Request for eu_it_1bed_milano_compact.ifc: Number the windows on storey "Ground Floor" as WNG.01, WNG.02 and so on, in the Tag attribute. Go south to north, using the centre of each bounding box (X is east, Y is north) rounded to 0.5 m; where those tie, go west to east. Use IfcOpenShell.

First a look at what the model holds.

```python
import ifcopenshell
import ifcopenshell.util.element
import ifcopenshell.util.placement

model = ifcopenshell.open("eu_it_1bed_milano_compact.ifc")
print(model.schema)
storey = next(s for s in model.by_type("IfcBuildingStorey") if s.Name == "Ground Floor")
windows = [e for e in ifcopenshell.util.element.get_decomposition(storey) if e.is_a("IfcWindow")]
for e in sorted(windows, key=lambda e: e.id()):
    origin = ifcopenshell.util.placement.get_local_placement(e.ObjectPlacement)[:3, 3]
    print(e.id(), e.Tag, e.Name, origin.round(2) + 0.0, sep=" | ")
```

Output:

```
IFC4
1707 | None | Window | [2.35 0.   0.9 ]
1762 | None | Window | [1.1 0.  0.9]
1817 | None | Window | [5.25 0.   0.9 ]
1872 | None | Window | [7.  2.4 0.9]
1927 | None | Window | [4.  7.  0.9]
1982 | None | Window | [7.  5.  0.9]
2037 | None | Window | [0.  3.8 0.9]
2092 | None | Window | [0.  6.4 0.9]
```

```python
import ifcopenshell
import ifcopenshell.geom
import ifcopenshell.util.element
import ifcopenshell.util.shape

model = ifcopenshell.open("eu_it_1bed_milano_compact.ifc")
settings = ifcopenshell.geom.settings()
settings.set("use-world-coords", True)


def centre(element):
    shape = ifcopenshell.geom.create_shape(settings, element)
    return ifcopenshell.util.shape.get_bbox_centroid(shape.geometry)


storey = next(s for s in model.by_type("IfcBuildingStorey") if s.Name == "Ground Floor")
windows = [e for e in ifcopenshell.util.element.get_decomposition(storey) if e.is_a("IfcWindow")]

# Insertion points can sit at a corner or the storey origin, so sort by the geometry (in metres).
centres = {e: centre(e) for e in windows}
windows.sort(key=lambda e: (round(centres[e][1] / 0.5), centres[e][0]))

for i, e in enumerate(windows, start=1):
    number = f"WNG.{i:02d}"
    e.Tag = number
    print(e.id(), number)

model.write("eu_it_1bed_milano_compact_edited.ifc")
```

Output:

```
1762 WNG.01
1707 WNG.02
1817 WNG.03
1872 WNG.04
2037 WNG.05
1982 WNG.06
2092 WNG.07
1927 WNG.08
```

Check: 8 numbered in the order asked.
